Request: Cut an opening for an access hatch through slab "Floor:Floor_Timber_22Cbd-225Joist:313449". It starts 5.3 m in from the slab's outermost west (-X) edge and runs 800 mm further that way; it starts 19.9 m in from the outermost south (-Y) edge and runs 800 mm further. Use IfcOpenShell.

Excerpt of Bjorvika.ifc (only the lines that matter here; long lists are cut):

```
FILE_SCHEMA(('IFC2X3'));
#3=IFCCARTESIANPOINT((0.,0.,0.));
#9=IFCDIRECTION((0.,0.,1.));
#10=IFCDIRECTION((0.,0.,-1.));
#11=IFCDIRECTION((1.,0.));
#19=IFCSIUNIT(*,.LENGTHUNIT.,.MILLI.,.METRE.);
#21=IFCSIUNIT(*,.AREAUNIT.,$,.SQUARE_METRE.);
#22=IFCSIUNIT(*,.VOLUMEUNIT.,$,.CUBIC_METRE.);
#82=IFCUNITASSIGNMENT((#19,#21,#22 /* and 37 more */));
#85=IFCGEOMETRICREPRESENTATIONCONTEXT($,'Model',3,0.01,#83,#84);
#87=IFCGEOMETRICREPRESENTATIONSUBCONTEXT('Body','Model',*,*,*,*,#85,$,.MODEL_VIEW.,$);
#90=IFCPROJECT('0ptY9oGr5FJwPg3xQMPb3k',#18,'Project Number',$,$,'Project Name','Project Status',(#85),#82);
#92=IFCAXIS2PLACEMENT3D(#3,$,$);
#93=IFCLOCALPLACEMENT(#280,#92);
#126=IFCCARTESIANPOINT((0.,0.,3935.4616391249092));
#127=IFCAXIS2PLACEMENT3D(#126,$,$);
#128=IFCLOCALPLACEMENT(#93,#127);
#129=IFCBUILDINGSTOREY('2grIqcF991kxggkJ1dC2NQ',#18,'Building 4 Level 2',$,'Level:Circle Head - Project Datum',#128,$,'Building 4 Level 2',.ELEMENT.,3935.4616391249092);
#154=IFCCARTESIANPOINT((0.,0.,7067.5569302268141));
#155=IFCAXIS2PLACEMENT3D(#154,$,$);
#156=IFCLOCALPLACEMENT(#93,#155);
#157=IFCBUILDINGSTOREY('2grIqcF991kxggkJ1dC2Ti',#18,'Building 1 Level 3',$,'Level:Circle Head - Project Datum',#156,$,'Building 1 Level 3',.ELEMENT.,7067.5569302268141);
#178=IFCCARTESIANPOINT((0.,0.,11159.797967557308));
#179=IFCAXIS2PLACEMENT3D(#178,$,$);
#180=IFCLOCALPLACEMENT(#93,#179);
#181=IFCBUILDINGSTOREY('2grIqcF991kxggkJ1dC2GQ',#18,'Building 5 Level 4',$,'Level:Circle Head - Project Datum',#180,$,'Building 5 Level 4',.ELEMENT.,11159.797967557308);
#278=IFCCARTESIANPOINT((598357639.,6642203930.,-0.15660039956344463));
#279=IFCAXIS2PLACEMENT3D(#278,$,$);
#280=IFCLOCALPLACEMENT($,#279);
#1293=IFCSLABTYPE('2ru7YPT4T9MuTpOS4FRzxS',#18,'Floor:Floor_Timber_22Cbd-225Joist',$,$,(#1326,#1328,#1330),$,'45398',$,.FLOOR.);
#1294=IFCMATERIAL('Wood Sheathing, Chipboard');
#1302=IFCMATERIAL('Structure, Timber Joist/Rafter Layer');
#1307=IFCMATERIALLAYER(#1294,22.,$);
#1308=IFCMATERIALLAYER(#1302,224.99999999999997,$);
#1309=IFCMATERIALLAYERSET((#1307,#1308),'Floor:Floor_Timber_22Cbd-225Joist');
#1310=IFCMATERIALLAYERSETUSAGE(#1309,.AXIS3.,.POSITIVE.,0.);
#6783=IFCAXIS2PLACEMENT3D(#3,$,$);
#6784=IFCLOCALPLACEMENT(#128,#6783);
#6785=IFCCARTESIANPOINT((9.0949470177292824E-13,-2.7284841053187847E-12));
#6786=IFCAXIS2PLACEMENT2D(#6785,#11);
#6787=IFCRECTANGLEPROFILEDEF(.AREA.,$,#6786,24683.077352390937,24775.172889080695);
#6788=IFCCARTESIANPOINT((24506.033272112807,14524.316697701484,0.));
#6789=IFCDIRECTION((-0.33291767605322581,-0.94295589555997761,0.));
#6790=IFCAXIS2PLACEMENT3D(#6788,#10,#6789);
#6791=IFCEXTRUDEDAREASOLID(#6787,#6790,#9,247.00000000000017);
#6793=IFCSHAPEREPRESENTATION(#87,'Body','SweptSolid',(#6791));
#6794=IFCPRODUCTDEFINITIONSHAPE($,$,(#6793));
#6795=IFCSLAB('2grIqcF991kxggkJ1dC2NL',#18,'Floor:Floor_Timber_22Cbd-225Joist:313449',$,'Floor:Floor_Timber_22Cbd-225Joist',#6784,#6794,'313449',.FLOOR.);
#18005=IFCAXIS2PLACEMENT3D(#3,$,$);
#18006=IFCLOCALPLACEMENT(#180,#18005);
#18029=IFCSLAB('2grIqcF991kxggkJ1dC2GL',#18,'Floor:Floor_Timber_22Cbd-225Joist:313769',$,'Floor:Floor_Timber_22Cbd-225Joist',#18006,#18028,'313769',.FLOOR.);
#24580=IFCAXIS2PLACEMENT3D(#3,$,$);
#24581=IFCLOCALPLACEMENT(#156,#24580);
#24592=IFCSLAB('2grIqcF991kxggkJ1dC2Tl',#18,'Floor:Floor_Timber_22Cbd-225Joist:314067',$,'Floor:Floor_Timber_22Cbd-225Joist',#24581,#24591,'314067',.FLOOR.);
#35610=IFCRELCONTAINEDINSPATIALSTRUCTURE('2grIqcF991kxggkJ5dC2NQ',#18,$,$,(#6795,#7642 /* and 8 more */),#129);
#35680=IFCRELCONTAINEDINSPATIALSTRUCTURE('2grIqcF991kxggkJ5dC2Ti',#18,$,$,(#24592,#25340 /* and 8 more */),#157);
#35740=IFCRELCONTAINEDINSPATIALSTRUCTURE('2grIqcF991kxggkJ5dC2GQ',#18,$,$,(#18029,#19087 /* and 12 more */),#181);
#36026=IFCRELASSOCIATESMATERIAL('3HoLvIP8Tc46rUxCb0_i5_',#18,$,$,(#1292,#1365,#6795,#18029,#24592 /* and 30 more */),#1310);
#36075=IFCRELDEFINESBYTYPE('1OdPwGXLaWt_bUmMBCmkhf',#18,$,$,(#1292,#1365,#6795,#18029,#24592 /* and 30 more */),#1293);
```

```python
import numpy as np
import ifcopenshell
import ifcopenshell.api.feature
import ifcopenshell.api.geometry
import ifcopenshell.api.root
import ifcopenshell.geom
import ifcopenshell.util.placement
import ifcopenshell.util.representation
import ifcopenshell.util.shape
import ifcopenshell.util.unit

model = ifcopenshell.open("Bjorvika.ifc")
unit_scale = ifcopenshell.util.unit.calculate_unit_scale(model)
settings = ifcopenshell.geom.settings()


def volume(element):
    """Net volume in cubic metres, openings subtracted."""
    shape = ifcopenshell.geom.create_shape(settings, element)
    return ifcopenshell.util.shape.get_volume(shape.geometry)


slab = model.by_id(6795)
before = volume(slab)

# Extent in the slab's own axes, in metres. The edges named are its -X and -Y sides.
slab_shape = ifcopenshell.geom.create_shape(settings, slab)
vertices = ifcopenshell.util.shape.get_vertices(slab_shape.geometry)
x_min, y_min, bottom = vertices.min(axis=0)
top = vertices[:, 2].max()

opening = ifcopenshell.api.root.create_entity(model, ifc_class="IfcOpeningElement", name="Access hatch opening")
context = ifcopenshell.util.representation.get_context(model, "Model", "Body", "MODEL_VIEW")
width, depth = 0.8, 0.8
outline = [(0.0, 0.0), (width, 0.0), (width, depth), (0.0, depth), (0.0, 0.0)]
# Overshoot both faces by 50 mm so the cut is clean.
shape = ifcopenshell.api.geometry.add_slab_representation(
    model, context=context, depth=top - bottom + 0.1, polyline=outline
)
ifcopenshell.api.geometry.assign_representation(model, product=opening, representation=shape)

matrix = ifcopenshell.util.placement.get_local_placement(slab.ObjectPlacement)
matrix[:, 3] = matrix @ np.append(np.array([x_min + 5.3, y_min + 19.9, bottom - 0.05]) / unit_scale, 1.0)
ifcopenshell.api.geometry.edit_object_placement(model, product=opening, matrix=matrix, is_si=False)
ifcopenshell.api.feature.add_feature(model, feature=opening, element=slab)

after = volume(slab)

print(f"slab volume {before:.3f} -> {after:.3f} m3")

model.write("Bjorvika_rev.ifc")
```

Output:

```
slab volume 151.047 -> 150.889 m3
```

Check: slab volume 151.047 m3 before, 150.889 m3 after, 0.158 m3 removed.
